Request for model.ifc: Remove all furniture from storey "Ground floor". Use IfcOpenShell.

First a look at what the model holds.

```python
import ifcopenshell
import ifcopenshell.util.element

model = ifcopenshell.open("model.ifc")
print(model.schema)
storey = next(s for s in model.by_type("IfcBuildingStorey") if s.Name == "Ground floor")
furniture = [e for e in ifcopenshell.util.element.get_decomposition(storey) if e.is_a("IfcFurnishingElement")]
seen = {}
for e in furniture:
    element_type = ifcopenshell.util.element.get_type(e)
    name = element_type.Name if element_type not in (None, e) else None
    seen[name] = seen.get(name, 0) + 1
for name, count in sorted(seen.items(), key=str):
    print(count, "x", name)
```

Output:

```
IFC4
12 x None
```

```python
import ifcopenshell
import ifcopenshell.api.root
import ifcopenshell.util.element

model = ifcopenshell.open("model.ifc")

storey = next(s for s in model.by_type("IfcBuildingStorey") if s.Name == "Ground floor")
furniture = [e for e in ifcopenshell.util.element.get_decomposition(storey) if e.is_a("IfcFurnishingElement")]

for e in furniture:
    ifcopenshell.api.root.remove_product(model, product=e)
print(len(furniture), "removed")

model.write("model-out.ifc")
```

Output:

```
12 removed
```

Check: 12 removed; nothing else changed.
